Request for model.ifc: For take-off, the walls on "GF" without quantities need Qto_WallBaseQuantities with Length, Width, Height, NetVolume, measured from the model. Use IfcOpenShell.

First a look at what the model holds.

```python
import ifcopenshell
import ifcopenshell.util.element
import ifcopenshell.util.unit

model = ifcopenshell.open("model.ifc")
print(model.schema)
for unit_type in ("LENGTHUNIT", "AREAUNIT", "VOLUMEUNIT"):
    print(unit_type, ifcopenshell.util.unit.calculate_unit_scale(model, unit_type))
storey = next(s for s in model.by_type("IfcBuildingStorey") if s.Name == "GF")
walls = [e for e in ifcopenshell.util.element.get_decomposition(storey) if e.is_a("IfcWall")]
for e in sorted(walls, key=lambda e: e.id()):
    print(e.id(), e.is_a(), e.Name, list(ifcopenshell.util.element.get_psets(e, qtos_only=True)), sep=" | ")
```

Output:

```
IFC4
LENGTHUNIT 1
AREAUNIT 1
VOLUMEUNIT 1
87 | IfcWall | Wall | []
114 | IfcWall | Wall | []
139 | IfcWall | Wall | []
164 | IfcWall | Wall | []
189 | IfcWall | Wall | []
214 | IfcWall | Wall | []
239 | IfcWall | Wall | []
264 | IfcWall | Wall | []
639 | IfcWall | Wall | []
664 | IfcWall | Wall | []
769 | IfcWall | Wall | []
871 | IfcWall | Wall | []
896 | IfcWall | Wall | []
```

```python
import ifcopenshell
import ifcopenshell.api.pset
import ifcopenshell.geom
import ifcopenshell.util.element
import ifcopenshell.util.shape
import ifcopenshell.util.unit

model = ifcopenshell.open("model.ifc")
unit_scale = ifcopenshell.util.unit.calculate_unit_scale(model)
volume_scale = ifcopenshell.util.unit.calculate_unit_scale(model, "VOLUMEUNIT")
settings = ifcopenshell.geom.settings()

storey = next(s for s in model.by_type("IfcBuildingStorey") if s.Name == "GF")
walls = [e for e in ifcopenshell.util.element.get_decomposition(storey) if e.is_a("IfcWall")]

for e in sorted(walls, key=lambda e: e.id()):
    if ifcopenshell.util.element.get_psets(e, qtos_only=True, should_inherit=False):
        continue
    # Geometry comes back in metres, in the element's own axes.
    shape = ifcopenshell.geom.create_shape(settings, e)
    values = {
        "Length": ifcopenshell.util.shape.get_x(shape.geometry) / unit_scale,
        "Width": ifcopenshell.util.shape.get_y(shape.geometry) / unit_scale,
        "Height": ifcopenshell.util.shape.get_z(shape.geometry) / unit_scale,
        "NetVolume": ifcopenshell.util.shape.get_volume(shape.geometry) / volume_scale,
    }
    qto = ifcopenshell.api.pset.add_qto(model, product=e, name="Qto_WallBaseQuantities")
    ifcopenshell.api.pset.edit_qto(model, qto=qto, properties=values)
    print(e.id(), {k: round(v, 3) for k, v in values.items()})

model.write("model-out.ifc")
```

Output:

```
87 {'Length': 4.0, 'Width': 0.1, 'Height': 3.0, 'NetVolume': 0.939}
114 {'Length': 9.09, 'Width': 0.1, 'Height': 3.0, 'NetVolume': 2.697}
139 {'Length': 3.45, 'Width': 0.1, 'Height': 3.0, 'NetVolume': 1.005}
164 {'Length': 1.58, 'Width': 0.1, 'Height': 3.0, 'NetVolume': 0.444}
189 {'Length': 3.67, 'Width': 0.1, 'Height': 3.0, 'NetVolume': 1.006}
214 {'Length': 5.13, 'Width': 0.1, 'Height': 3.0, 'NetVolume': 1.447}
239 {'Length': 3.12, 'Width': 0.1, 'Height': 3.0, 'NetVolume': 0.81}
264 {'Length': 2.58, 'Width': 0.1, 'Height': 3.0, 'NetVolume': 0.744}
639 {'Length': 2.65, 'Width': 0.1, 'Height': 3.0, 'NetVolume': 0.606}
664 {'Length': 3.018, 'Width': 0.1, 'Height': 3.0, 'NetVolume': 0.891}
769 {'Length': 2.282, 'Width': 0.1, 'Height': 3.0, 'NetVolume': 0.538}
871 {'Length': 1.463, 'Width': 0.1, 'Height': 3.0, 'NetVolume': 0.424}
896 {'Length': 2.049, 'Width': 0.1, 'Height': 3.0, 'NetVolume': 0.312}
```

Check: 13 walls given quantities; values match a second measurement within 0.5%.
